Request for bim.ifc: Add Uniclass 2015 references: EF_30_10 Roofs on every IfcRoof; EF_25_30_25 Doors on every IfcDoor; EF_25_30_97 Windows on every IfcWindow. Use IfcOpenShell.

First a look at what the model holds.

```python
import ifcopenshell

model = ifcopenshell.open("bim.ifc")
print(model.schema)
print("classifications:", [c.Name for c in model.by_type("IfcClassification")])
for ifc_class in ("IfcDoor", "IfcRoof", "IfcStair", "IfcWall", "IfcWindow"):
    print(ifc_class, len(model.by_type(ifc_class)))
```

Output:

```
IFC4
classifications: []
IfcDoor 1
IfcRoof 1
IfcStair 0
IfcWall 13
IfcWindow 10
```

```python
import ifcopenshell
import ifcopenshell.api.classification

model = ifcopenshell.open("bim.ifc")

system = ifcopenshell.api.classification.add_classification(model, classification="Uniclass 2015")

codes = {
    "IfcRoof": ("EF_30_10", "Roofs"),
    "IfcDoor": ("EF_25_30_25", "Doors"),
    "IfcWindow": ("EF_25_30_97", "Windows"),
}
for ifc_class, (code, name) in codes.items():
    products = model.by_type(ifc_class)
    ifcopenshell.api.classification.add_reference(
        model, products=products, classification=system, identification=code, name=name
    )
    print(code, len(products))

model.write("bim_v2.ifc")
```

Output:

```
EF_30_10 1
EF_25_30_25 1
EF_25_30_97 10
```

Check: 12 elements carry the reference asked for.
